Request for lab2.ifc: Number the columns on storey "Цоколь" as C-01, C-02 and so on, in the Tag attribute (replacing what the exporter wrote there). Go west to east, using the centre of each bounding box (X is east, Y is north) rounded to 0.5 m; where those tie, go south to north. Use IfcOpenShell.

First a look at what the model holds.

```python
import ifcopenshell
import ifcopenshell.util.element
import ifcopenshell.util.placement

model = ifcopenshell.open("lab2.ifc")
print(model.schema)
storey = next(s for s in model.by_type("IfcBuildingStorey") if s.Name == "Цоколь")
columns = [e for e in ifcopenshell.util.element.get_decomposition(storey) if e.is_a("IfcColumn")]
for e in sorted(columns, key=lambda e: e.id()):
    origin = ifcopenshell.util.placement.get_local_placement(e.ObjectPlacement)[:3, 3]
    print(e.id(), e.Tag, e.Name, origin.round(2) + 0.0, sep=" | ")
```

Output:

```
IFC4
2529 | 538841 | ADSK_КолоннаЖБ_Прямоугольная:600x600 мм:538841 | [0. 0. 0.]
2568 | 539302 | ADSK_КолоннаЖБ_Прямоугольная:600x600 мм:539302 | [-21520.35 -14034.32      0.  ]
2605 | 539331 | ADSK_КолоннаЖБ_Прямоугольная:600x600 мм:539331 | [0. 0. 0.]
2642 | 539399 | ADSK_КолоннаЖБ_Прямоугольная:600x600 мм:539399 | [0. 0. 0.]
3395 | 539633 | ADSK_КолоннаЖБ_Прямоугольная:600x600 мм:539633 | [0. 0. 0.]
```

```python
import ifcopenshell
import ifcopenshell.geom
import ifcopenshell.util.element
import ifcopenshell.util.shape

model = ifcopenshell.open("lab2.ifc")
settings = ifcopenshell.geom.settings()
settings.set("use-world-coords", True)


def centre(element):
    shape = ifcopenshell.geom.create_shape(settings, element)
    return ifcopenshell.util.shape.get_bbox_centroid(shape.geometry)


storey = next(s for s in model.by_type("IfcBuildingStorey") if s.Name == "Цоколь")
columns = [e for e in ifcopenshell.util.element.get_decomposition(storey) if e.is_a("IfcColumn")]

# Insertion points can sit at a corner or the storey origin, so sort by the geometry (in metres).
centres = {e: centre(e) for e in columns}
columns.sort(key=lambda e: (round(centres[e][0] / 0.5), centres[e][1]))

for i, e in enumerate(columns, start=1):
    number = f"C-{i:02d}"
    e.Tag = number
    print(e.id(), number)

model.write("lab2-out.ifc")
```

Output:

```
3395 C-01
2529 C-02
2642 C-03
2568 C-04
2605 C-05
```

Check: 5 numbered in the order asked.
